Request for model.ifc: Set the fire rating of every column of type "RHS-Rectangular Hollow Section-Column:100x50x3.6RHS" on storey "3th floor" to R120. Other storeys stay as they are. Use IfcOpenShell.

First a look at what the model holds.

```python
import ifcopenshell
import ifcopenshell.util.element

model = ifcopenshell.open("model.ifc")
print(model.schema)
storey = next(s for s in model.by_type("IfcBuildingStorey") if s.Name == "3th floor")
columns = [e for e in ifcopenshell.util.element.get_decomposition(storey) if e.is_a("IfcColumn")]
seen = {}
for e in columns:
    element_type = ifcopenshell.util.element.get_type(e)
    key = (element_type.Name if element_type != e and element_type else None, ifcopenshell.util.element.get_pset(e, "Pset_ColumnCommon", "FireRating"))
    seen[key] = seen.get(key, 0) + 1
for (name, value), count in sorted(seen.items(), key=str):
    print(count, "x", name, "|", value)
```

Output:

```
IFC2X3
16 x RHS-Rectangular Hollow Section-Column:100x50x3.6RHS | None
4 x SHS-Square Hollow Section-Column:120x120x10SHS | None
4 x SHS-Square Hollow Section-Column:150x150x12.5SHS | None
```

```python
import ifcopenshell
import ifcopenshell.api.pset
import ifcopenshell.util.element

model = ifcopenshell.open("model.ifc")

storey = next(s for s in model.by_type("IfcBuildingStorey") if s.Name == "3th floor")
columns = [e for e in ifcopenshell.util.element.get_decomposition(storey) if e.is_a("IfcColumn")]

count = 0
for e in columns:
    element_type = ifcopenshell.util.element.get_type(e)
    if element_type in (None, e) or element_type.Name != "RHS-Rectangular Hollow Section-Column:100x50x3.6RHS":
        continue
    # add_pset returns the element's existing set when there is one.
    pset = ifcopenshell.api.pset.add_pset(model, product=e, name="Pset_ColumnCommon")
    ifcopenshell.api.pset.edit_pset(model, pset=pset, properties={"FireRating": "R120"})
    count += 1

print(count, "columns updated")

model.write("model-out.ifc")
```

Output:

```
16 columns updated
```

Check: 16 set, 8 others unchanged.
